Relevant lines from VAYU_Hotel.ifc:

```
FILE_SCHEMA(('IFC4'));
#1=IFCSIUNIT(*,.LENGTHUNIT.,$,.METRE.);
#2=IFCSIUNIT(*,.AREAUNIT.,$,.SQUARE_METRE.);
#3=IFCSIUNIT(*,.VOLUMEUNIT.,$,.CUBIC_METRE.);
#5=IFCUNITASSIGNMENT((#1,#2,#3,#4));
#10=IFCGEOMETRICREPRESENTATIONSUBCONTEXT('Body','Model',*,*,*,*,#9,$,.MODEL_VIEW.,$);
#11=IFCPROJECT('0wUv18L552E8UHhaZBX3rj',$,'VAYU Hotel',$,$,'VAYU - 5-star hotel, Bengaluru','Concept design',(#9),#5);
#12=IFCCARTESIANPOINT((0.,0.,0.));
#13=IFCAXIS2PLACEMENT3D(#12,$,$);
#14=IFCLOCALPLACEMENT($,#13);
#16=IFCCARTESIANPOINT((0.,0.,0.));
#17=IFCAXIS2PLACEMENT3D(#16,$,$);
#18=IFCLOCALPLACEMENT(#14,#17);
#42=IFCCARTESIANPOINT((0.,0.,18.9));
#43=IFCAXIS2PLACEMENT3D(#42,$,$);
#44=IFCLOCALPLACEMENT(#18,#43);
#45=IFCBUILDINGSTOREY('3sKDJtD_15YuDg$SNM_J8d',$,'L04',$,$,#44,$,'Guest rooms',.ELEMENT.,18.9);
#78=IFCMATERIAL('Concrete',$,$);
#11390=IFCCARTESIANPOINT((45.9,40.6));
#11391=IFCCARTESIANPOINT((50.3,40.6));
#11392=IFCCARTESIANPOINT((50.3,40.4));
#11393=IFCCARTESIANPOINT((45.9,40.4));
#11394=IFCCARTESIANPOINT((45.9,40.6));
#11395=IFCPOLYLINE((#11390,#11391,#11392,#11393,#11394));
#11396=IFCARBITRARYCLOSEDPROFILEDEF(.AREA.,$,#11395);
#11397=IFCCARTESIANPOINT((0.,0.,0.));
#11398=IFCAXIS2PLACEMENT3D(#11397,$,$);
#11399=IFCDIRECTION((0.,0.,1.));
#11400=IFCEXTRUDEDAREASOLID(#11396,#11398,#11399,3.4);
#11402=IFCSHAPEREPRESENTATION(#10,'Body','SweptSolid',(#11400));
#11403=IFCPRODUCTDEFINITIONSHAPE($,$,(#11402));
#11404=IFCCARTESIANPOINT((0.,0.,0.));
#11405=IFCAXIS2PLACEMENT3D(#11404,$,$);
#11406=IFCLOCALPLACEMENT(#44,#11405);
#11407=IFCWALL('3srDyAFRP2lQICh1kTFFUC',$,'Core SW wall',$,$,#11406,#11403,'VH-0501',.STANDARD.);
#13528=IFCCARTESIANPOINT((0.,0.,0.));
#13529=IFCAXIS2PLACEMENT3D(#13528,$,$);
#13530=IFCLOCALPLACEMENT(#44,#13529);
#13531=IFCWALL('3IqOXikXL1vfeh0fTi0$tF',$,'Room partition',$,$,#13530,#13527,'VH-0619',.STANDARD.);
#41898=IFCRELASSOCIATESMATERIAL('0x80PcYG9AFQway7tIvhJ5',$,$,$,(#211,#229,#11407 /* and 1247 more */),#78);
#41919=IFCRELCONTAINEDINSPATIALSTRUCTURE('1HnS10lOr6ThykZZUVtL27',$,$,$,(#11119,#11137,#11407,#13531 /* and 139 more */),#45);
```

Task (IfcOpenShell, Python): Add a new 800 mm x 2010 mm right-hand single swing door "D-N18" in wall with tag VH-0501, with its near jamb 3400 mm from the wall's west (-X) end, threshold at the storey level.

```python
import numpy as np
import ifcopenshell
import ifcopenshell.api.feature
import ifcopenshell.api.geometry
import ifcopenshell.api.root
import ifcopenshell.api.spatial
import ifcopenshell.geom
import ifcopenshell.util.element
import ifcopenshell.util.placement
import ifcopenshell.util.representation
import ifcopenshell.util.shape
import ifcopenshell.util.unit

model = ifcopenshell.open("VAYU_Hotel.ifc")
unit_scale = ifcopenshell.util.unit.calculate_unit_scale(model)
settings = ifcopenshell.geom.settings()


def volume(element):
    """Net volume in cubic metres, openings subtracted."""
    shape = ifcopenshell.geom.create_shape(settings, element)
    return ifcopenshell.util.shape.get_volume(shape.geometry)


wall = model.by_id(11407)
storey = ifcopenshell.util.element.get_container(wall, ifc_class="IfcBuildingStorey")
context = ifcopenshell.util.representation.get_context(model, "Model", "Body", "MODEL_VIEW")
before = volume(wall)

width, height, from_end, sill = 0.8, 2.01, 3.4, 0.0  # metres

# The wall runs along its own X axis, and the end named is its -X end.
wall_shape = ifcopenshell.geom.create_shape(settings, wall)
x, y, z = ifcopenshell.util.shape.get_vertices(wall_shape.geometry).T
start = x.min() + from_end
face, thickness = float(y.min()), float(y.max() - y.min())
wall_matrix = ifcopenshell.util.placement.get_local_placement(wall.ObjectPlacement)
level = ifcopenshell.util.placement.get_local_placement(storey.ObjectPlacement)[2, 3]


def in_wall(x, y):
    """Placement at x, y metres in the wall's axes, at sill height."""
    matrix = wall_matrix.copy()
    matrix[:, 3] = wall_matrix @ np.array([x / unit_scale, y / unit_scale, 0.0, 1.0])
    matrix[2, 3] = level + sill / unit_scale
    return matrix


# Opening: a box that overshoots both wall faces by 50 mm.
opening = ifcopenshell.api.root.create_entity(model, ifc_class="IfcOpeningElement", predefined_type="OPENING")
box = ifcopenshell.api.geometry.add_wall_representation(
    model, context=context, length=width, height=height, thickness=thickness + 0.1
)
ifcopenshell.api.geometry.assign_representation(model, product=opening, representation=box)
ifcopenshell.api.geometry.edit_object_placement(model, product=opening, matrix=in_wall(start, face - 0.05), is_si=False)
ifcopenshell.api.feature.add_feature(model, feature=opening, element=wall)

door = ifcopenshell.api.root.create_entity(model, ifc_class="IfcDoor", name="D-N18", predefined_type="DOOR")
door.OverallWidth, door.OverallHeight = width / unit_scale, height / unit_scale
door.OperationType = "SINGLE_SWING_RIGHT"
body = ifcopenshell.api.geometry.add_door_representation(
    model,
    context=context,
    overall_width=door.OverallWidth,
    overall_height=door.OverallHeight,
    operation_type="SINGLE_SWING_RIGHT",
    lining_properties={"LiningDepth": thickness / unit_scale, "ThresholdDepth": thickness / unit_scale},
)
ifcopenshell.api.geometry.assign_representation(model, product=door, representation=body)
ifcopenshell.api.spatial.assign_container(model, products=[door], relating_structure=storey)
ifcopenshell.api.feature.add_filling(model, opening=opening, element=door)

# The lining spans the wall, so the door starts at the wall face.
ifcopenshell.api.geometry.edit_object_placement(model, product=door, matrix=in_wall(start, face), is_si=False)

after = volume(wall)

print(f"wall volume {before:.3f} -> {after:.3f} m3")

model.write("VAYU_Hotel_edited.ifc")
```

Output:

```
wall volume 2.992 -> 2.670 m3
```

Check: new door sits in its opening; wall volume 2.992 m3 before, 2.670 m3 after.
